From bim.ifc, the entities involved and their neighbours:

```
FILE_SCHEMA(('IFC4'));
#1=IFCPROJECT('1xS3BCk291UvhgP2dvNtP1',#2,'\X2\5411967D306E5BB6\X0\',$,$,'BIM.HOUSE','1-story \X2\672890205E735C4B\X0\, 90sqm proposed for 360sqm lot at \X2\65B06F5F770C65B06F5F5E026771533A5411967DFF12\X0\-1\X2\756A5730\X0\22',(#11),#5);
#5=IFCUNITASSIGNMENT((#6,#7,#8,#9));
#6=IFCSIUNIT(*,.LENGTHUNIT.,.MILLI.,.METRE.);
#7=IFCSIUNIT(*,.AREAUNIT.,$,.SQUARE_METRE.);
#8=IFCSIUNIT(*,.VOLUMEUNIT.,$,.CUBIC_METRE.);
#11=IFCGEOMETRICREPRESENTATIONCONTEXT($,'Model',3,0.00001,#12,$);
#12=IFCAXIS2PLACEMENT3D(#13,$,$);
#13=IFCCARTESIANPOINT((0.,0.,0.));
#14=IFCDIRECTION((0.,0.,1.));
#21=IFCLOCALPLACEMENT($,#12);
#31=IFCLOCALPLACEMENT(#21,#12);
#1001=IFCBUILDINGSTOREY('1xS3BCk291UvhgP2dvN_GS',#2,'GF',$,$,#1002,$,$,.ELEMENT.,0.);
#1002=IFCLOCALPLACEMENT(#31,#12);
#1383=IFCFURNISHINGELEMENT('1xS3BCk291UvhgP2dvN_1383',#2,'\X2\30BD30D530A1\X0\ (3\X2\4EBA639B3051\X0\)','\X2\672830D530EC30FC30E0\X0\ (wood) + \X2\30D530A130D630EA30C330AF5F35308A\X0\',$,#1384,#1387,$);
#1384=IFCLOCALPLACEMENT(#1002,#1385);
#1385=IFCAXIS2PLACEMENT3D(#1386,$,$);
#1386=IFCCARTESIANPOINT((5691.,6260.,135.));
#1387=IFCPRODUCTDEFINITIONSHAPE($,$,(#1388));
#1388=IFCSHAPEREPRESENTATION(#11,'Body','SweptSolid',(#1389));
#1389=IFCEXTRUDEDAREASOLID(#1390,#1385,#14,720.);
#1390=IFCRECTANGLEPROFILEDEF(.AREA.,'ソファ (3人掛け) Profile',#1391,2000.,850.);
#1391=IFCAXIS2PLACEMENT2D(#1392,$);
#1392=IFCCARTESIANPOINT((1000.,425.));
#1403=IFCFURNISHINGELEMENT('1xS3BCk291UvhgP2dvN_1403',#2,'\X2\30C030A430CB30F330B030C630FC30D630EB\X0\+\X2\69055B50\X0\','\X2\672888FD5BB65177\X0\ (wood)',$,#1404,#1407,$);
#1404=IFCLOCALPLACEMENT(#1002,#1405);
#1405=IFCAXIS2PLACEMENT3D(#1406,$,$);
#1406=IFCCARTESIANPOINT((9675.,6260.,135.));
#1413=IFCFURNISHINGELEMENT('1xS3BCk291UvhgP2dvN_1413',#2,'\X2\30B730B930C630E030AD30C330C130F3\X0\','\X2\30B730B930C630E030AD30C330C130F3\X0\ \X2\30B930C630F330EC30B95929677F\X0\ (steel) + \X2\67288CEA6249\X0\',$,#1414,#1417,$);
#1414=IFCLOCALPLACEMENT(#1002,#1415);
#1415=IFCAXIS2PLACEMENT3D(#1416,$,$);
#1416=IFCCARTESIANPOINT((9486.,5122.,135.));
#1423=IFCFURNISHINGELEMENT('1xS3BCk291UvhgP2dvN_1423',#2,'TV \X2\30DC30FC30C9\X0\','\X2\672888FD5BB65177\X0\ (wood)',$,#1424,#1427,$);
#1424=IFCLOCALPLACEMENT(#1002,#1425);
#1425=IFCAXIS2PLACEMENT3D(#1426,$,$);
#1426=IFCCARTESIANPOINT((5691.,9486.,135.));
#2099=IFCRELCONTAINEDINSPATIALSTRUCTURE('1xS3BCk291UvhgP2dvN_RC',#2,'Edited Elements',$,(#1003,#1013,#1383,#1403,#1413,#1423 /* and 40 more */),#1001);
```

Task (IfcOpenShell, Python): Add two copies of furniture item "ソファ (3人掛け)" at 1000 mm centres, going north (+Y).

```python
import numpy as np
import ifcopenshell
import ifcopenshell.api.geometry
import ifcopenshell.api.root
import ifcopenshell.util.element
import ifcopenshell.util.placement
import ifcopenshell.util.unit

model = ifcopenshell.open("bim.ifc")
unit_scale = ifcopenshell.util.unit.calculate_unit_scale(model)


def reuse_history(source, copy):
    """copy_class also copies each property set's owner history, people and application; keep the originals."""
    for rel in copy.IsDefinedBy:
        if rel.is_a("IfcRelDefinesByProperties") and (history := rel.RelatingPropertyDefinition.OwnerHistory):
            rel.RelatingPropertyDefinition.OwnerHistory = source.OwnerHistory
            ifcopenshell.util.element.remove_deep2(model, history)


source = model.by_guid("1xS3BCk291UvhgP2dvN_1383")
base = ifcopenshell.util.placement.get_local_placement(source.ObjectPlacement)
step = np.array([0.0, 1.0, 0.0]) * 1 / unit_scale

for i in range(1, 3):
    copy = ifcopenshell.api.root.copy_class(model, product=source)
    copy.Representation = ifcopenshell.util.element.copy_deep(
        model, source.Representation, exclude=["IfcGeometricRepresentationContext", "IfcRepresentationMap"]
    )
    reuse_history(source, copy)
    matrix = base.copy()
    matrix[:3, 3] += i * step
    print("added at", matrix[:3, 3].round(3) + 0.0)
    ifcopenshell.api.geometry.edit_object_placement(model, product=copy, matrix=matrix, is_si=False)

model.write("bim_edited.ifc")
```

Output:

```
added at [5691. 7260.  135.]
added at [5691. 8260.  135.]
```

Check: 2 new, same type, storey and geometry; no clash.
